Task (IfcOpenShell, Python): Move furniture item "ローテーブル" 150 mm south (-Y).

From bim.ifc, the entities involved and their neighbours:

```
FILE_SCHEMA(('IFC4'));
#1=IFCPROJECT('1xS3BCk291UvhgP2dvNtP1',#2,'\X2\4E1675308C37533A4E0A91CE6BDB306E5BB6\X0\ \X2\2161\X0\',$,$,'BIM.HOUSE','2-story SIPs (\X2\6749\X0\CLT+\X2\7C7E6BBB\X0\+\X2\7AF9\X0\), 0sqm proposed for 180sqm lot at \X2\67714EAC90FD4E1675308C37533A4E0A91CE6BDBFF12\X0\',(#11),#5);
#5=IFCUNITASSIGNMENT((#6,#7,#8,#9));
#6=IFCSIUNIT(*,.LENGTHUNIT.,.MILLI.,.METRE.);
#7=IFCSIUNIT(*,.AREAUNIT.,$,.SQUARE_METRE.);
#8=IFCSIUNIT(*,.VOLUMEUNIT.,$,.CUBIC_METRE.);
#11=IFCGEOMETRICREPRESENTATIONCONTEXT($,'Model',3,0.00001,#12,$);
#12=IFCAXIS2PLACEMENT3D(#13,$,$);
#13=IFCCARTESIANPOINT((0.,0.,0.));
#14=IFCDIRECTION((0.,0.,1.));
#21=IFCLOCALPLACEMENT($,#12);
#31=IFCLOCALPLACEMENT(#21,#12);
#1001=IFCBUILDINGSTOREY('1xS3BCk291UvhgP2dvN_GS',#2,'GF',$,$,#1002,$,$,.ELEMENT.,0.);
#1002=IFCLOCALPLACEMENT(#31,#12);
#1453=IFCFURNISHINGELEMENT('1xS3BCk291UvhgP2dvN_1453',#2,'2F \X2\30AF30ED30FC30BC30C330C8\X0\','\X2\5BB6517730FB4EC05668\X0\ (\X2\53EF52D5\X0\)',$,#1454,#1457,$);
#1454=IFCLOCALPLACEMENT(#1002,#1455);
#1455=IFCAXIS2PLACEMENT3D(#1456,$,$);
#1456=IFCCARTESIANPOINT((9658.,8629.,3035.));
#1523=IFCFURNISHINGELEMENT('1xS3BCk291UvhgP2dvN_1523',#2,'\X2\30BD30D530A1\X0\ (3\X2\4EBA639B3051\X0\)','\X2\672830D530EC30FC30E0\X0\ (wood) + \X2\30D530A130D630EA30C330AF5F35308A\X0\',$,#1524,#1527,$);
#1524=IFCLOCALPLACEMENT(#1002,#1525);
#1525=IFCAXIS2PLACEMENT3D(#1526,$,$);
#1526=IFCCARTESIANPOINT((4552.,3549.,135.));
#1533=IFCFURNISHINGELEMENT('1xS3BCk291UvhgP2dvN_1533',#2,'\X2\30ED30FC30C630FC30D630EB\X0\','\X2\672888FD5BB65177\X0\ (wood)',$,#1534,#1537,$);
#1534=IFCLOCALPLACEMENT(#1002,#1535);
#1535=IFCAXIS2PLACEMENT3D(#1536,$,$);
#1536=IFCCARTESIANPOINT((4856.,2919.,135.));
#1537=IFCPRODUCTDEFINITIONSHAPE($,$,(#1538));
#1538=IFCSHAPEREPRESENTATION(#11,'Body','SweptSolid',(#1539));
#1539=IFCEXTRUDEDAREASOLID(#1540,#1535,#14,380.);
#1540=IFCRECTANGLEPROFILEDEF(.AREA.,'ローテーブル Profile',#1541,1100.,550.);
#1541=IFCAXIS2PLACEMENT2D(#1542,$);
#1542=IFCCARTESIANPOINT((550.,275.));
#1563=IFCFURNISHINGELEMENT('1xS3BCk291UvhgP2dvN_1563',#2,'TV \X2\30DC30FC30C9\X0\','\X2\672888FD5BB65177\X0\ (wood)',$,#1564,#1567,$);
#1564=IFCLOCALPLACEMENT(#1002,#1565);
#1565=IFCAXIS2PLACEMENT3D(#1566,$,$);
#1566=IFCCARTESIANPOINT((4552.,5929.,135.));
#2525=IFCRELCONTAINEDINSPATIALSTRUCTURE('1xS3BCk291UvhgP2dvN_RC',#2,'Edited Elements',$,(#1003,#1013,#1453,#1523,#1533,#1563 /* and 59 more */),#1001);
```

```python
import ifcopenshell
import ifcopenshell.api.geometry
import ifcopenshell.util.placement
import ifcopenshell.util.unit

model = ifcopenshell.open("bim.ifc")
unit_scale = ifcopenshell.util.unit.calculate_unit_scale(model)

item = model.by_guid("1xS3BCk291UvhgP2dvN_1533")
matrix = ifcopenshell.util.placement.get_local_placement(item.ObjectPlacement)
matrix[1, 3] -= 0.15 / unit_scale
ifcopenshell.api.geometry.edit_object_placement(model, product=item, matrix=matrix, is_si=False)

print(ifcopenshell.util.placement.get_local_placement(item.ObjectPlacement).round(3) + 0.0)

model.write("bim_updated.ifc")
```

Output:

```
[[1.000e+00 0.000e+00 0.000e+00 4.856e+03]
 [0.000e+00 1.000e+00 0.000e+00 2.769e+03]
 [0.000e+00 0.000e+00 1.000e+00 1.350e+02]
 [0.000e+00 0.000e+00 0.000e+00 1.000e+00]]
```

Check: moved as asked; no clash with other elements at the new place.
